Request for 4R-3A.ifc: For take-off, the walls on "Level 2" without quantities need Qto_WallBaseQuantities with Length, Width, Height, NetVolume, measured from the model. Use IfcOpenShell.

First a look at what the model holds.

```python
import ifcopenshell
import ifcopenshell.util.element
import ifcopenshell.util.unit

model = ifcopenshell.open("4R-3A.ifc")
print(model.schema)
for unit_type in ("LENGTHUNIT", "AREAUNIT", "VOLUMEUNIT"):
    print(unit_type, ifcopenshell.util.unit.calculate_unit_scale(model, unit_type))
storey = next(s for s in model.by_type("IfcBuildingStorey") if s.Name == "Level 2")
walls = [e for e in ifcopenshell.util.element.get_decomposition(storey) if e.is_a("IfcWall")]
for e in sorted(walls, key=lambda e: e.id()):
    print(e.id(), e.is_a(), e.Name, list(ifcopenshell.util.element.get_psets(e, qtos_only=True)), sep=" | ")
```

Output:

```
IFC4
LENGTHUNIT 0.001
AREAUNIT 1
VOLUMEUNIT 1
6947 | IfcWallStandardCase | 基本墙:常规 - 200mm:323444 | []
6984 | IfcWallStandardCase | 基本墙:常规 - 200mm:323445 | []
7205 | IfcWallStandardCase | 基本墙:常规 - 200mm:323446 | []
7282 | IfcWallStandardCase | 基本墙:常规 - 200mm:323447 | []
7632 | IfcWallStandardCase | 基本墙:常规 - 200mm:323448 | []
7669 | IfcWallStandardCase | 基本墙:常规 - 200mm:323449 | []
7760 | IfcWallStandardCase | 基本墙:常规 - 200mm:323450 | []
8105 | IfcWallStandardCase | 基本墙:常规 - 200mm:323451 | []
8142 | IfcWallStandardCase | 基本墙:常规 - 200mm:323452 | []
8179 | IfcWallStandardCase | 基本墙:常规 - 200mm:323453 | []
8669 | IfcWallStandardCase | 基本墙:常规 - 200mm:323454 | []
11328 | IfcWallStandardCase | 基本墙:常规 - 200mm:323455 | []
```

```python
import ifcopenshell
import ifcopenshell.api.pset
import ifcopenshell.geom
import ifcopenshell.util.element
import ifcopenshell.util.shape
import ifcopenshell.util.unit

model = ifcopenshell.open("4R-3A.ifc")
unit_scale = ifcopenshell.util.unit.calculate_unit_scale(model)
volume_scale = ifcopenshell.util.unit.calculate_unit_scale(model, "VOLUMEUNIT")
settings = ifcopenshell.geom.settings()

storey = next(s for s in model.by_type("IfcBuildingStorey") if s.Name == "Level 2")
walls = [e for e in ifcopenshell.util.element.get_decomposition(storey) if e.is_a("IfcWall")]

for e in sorted(walls, key=lambda e: e.id()):
    if ifcopenshell.util.element.get_psets(e, qtos_only=True, should_inherit=False):
        continue
    # Geometry comes back in metres, in the element's own axes.
    shape = ifcopenshell.geom.create_shape(settings, e)
    values = {
        "Length": ifcopenshell.util.shape.get_x(shape.geometry) / unit_scale,
        "Width": ifcopenshell.util.shape.get_y(shape.geometry) / unit_scale,
        "Height": ifcopenshell.util.shape.get_z(shape.geometry) / unit_scale,
        "NetVolume": ifcopenshell.util.shape.get_volume(shape.geometry) / volume_scale,
    }
    qto = ifcopenshell.api.pset.add_qto(model, product=e, name="Qto_WallBaseQuantities")
    ifcopenshell.api.pset.edit_qto(model, qto=qto, properties=values)
    print(e.id(), {k: round(v, 3) for k, v in values.items()})

model.write("4R-3A-out.ifc")
```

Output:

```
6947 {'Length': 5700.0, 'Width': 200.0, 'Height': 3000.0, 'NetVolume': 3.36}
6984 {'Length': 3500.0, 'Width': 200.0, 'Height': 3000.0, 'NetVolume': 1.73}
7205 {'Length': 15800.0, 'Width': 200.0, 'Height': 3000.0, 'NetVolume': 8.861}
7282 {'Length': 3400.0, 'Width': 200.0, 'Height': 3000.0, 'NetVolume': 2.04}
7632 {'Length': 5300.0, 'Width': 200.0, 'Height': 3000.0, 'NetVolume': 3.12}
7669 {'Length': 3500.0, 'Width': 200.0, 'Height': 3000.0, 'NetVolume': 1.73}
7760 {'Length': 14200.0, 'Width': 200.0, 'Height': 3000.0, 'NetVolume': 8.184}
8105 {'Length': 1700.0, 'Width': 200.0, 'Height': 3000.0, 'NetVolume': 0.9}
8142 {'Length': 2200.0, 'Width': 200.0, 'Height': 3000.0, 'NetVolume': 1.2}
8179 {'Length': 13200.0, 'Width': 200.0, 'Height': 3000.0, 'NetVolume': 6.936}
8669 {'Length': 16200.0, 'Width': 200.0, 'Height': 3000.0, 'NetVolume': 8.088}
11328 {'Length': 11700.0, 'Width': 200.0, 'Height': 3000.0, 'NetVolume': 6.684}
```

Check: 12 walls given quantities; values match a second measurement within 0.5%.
